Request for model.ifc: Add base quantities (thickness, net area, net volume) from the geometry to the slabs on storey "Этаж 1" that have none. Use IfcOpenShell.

First a look at what the model holds.

```python
import ifcopenshell
import ifcopenshell.util.element
import ifcopenshell.util.unit

model = ifcopenshell.open("model.ifc")
print(model.schema)
for unit_type in ("LENGTHUNIT", "AREAUNIT", "VOLUMEUNIT"):
    print(unit_type, ifcopenshell.util.unit.calculate_unit_scale(model, unit_type))
storey = next(s for s in model.by_type("IfcBuildingStorey") if s.Name == "Этаж 1")
slabs = [e for e in ifcopenshell.util.element.get_decomposition(storey) if e.is_a("IfcSlab")]
for e in sorted(slabs, key=lambda e: e.id()):
    print(e.id(), e.is_a(), e.Name, list(ifcopenshell.util.element.get_psets(e, qtos_only=True)), sep=" | ")
```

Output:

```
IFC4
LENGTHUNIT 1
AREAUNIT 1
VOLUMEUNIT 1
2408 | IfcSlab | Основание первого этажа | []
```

```python
import ifcopenshell
import ifcopenshell.api.pset
import ifcopenshell.geom
import ifcopenshell.util.element
import ifcopenshell.util.shape
import ifcopenshell.util.unit

model = ifcopenshell.open("model.ifc")
unit_scale = ifcopenshell.util.unit.calculate_unit_scale(model)
area_scale = ifcopenshell.util.unit.calculate_unit_scale(model, "AREAUNIT")
volume_scale = ifcopenshell.util.unit.calculate_unit_scale(model, "VOLUMEUNIT")
settings = ifcopenshell.geom.settings()

storey = next(s for s in model.by_type("IfcBuildingStorey") if s.Name == "Этаж 1")
slabs = [e for e in ifcopenshell.util.element.get_decomposition(storey) if e.is_a("IfcSlab")]

for e in sorted(slabs, key=lambda e: e.id()):
    if ifcopenshell.util.element.get_psets(e, qtos_only=True, should_inherit=False):
        continue
    # Geometry comes back in metres, in the element's own axes.
    shape = ifcopenshell.geom.create_shape(settings, e)
    values = {
        "Width": ifcopenshell.util.shape.get_z(shape.geometry) / unit_scale,
        "NetArea": ifcopenshell.util.shape.get_footprint_area(shape.geometry) / area_scale,
        "NetVolume": ifcopenshell.util.shape.get_volume(shape.geometry) / volume_scale,
    }
    qto = ifcopenshell.api.pset.add_qto(model, product=e, name="Qto_SlabBaseQuantities")
    ifcopenshell.api.pset.edit_qto(model, qto=qto, properties=values)
    print(e.id(), {k: round(v, 3) for k, v in values.items()})

model.write("model_updated.ifc")
```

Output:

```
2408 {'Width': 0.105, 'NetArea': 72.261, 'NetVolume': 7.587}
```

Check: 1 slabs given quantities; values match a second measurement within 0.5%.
